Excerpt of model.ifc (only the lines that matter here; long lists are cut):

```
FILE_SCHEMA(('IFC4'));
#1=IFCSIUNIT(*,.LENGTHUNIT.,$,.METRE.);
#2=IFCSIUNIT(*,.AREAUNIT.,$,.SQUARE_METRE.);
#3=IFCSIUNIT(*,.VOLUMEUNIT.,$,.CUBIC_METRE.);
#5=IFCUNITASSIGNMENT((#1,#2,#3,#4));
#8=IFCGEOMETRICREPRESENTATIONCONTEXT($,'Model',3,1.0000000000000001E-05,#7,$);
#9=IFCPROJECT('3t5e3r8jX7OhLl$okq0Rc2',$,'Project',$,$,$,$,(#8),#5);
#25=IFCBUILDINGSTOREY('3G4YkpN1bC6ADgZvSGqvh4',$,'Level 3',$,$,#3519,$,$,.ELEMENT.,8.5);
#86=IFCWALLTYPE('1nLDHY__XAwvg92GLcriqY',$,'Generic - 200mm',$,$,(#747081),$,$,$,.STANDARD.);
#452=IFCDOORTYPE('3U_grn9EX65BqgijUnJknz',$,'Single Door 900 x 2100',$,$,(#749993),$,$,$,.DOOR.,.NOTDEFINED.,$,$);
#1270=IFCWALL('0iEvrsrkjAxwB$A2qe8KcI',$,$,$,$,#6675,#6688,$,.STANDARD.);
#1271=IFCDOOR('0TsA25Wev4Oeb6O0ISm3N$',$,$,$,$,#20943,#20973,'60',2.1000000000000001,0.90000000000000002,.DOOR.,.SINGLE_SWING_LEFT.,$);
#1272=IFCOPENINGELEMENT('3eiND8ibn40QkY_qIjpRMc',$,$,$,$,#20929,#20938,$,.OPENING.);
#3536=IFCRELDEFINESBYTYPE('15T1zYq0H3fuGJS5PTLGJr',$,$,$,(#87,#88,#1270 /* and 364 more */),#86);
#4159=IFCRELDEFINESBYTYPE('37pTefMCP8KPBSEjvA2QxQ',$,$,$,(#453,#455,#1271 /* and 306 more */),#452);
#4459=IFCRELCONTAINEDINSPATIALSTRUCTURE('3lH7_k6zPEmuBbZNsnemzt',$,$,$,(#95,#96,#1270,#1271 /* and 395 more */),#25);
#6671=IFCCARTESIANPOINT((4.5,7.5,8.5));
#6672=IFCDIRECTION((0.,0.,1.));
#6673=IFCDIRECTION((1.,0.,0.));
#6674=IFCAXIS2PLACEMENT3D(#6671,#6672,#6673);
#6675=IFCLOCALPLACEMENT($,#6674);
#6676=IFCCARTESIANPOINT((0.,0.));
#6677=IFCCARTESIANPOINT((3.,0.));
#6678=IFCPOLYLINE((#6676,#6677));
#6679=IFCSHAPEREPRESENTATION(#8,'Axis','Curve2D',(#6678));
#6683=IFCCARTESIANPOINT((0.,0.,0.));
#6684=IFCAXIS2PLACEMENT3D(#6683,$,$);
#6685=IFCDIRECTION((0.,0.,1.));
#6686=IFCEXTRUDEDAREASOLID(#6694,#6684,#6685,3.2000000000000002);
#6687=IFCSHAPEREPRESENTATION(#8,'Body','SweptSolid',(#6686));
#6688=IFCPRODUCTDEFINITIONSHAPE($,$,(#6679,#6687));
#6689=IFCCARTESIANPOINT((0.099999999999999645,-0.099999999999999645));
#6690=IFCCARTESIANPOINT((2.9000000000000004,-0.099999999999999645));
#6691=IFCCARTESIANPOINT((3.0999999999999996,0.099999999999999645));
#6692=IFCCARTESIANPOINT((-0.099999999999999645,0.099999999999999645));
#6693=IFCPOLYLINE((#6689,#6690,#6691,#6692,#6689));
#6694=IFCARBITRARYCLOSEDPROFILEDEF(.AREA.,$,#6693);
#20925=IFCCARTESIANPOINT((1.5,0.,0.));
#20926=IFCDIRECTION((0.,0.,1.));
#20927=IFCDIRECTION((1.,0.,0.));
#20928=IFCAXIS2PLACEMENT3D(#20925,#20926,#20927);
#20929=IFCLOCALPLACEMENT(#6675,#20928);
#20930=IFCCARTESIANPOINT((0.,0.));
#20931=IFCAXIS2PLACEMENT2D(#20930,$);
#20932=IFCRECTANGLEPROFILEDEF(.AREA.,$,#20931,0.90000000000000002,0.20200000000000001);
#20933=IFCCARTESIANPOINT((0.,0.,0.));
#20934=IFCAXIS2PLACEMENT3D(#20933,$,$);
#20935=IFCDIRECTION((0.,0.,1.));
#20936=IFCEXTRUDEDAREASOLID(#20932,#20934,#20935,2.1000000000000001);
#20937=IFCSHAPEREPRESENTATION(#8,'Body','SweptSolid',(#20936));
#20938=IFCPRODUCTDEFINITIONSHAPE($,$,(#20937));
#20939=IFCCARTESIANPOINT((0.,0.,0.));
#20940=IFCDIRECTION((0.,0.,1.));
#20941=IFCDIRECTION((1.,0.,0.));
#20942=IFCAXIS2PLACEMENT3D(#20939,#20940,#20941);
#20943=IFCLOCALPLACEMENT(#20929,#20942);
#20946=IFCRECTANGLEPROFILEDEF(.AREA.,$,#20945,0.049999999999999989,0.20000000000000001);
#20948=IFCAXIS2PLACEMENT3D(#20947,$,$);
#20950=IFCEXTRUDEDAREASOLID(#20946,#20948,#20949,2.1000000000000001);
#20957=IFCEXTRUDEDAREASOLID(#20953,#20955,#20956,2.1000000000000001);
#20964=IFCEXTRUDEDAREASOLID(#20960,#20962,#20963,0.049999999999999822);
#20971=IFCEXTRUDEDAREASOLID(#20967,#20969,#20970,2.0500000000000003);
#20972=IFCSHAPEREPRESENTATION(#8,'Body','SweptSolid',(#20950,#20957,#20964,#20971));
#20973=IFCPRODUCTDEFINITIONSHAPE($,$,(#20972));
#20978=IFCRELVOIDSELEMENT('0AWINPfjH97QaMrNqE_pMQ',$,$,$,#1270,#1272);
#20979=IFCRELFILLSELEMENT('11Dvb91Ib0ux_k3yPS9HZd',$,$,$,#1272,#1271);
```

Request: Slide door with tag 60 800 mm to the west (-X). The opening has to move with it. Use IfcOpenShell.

```python
import ifcopenshell
import ifcopenshell.api.geometry
import ifcopenshell.util.placement

model = ifcopenshell.open("model.ifc")

door = model.by_guid("0TsA25Wev4Oeb6O0ISm3N$")
opening = door.FillsVoids[0].RelatingOpeningElement
wall = opening.VoidsElements[0].RelatingBuildingElement

wall_matrix = ifcopenshell.util.placement.get_local_placement(wall.ObjectPlacement)
shift = wall_matrix[:3, 0] * -0.8
before = ifcopenshell.util.placement.get_local_placement(door.ObjectPlacement)[:3, 3].copy()

# The door is placed relative to its opening, so it follows when the opening moves.
matrix = ifcopenshell.util.placement.get_local_placement(opening.ObjectPlacement)
matrix[:3, 3] += shift
ifcopenshell.api.geometry.edit_object_placement(
    model, product=opening, matrix=matrix, is_si=False, should_transform_children=True
)

after = ifcopenshell.util.placement.get_local_placement(door.ObjectPlacement)[:3, 3]
print("door moved by", (after - before).round(3) + 0.0)

model.write("model-out.ifc")
```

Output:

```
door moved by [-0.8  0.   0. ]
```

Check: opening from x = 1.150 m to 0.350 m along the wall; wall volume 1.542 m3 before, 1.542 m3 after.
